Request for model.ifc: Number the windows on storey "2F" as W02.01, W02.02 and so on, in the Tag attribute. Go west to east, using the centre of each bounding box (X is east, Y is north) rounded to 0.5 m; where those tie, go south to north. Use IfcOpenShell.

First a look at what the model holds.

```python
import ifcopenshell
import ifcopenshell.util.element
import ifcopenshell.util.placement

model = ifcopenshell.open("model.ifc")
print(model.schema)
storey = next(s for s in model.by_type("IfcBuildingStorey") if s.Name == "2F")
windows = [e for e in ifcopenshell.util.element.get_decomposition(storey) if e.is_a("IfcWindow")]
for e in sorted(windows, key=lambda e: e.id()):
    origin = ifcopenshell.util.placement.get_local_placement(e.ObjectPlacement)[:3, 3]
    print(e.id(), e.Tag, e.Name, origin.round(2) + 0.0, sep=" | ")
```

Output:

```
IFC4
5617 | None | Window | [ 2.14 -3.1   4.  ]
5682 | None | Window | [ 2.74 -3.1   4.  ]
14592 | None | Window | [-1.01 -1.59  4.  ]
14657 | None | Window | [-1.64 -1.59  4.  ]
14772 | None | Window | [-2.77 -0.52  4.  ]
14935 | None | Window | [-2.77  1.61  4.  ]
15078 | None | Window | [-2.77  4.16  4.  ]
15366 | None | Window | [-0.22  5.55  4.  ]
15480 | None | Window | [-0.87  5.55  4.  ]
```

```python
import ifcopenshell
import ifcopenshell.geom
import ifcopenshell.util.element
import ifcopenshell.util.shape

model = ifcopenshell.open("model.ifc")
settings = ifcopenshell.geom.settings()
settings.set("use-world-coords", True)


def centre(element):
    shape = ifcopenshell.geom.create_shape(settings, element)
    return ifcopenshell.util.shape.get_bbox_centroid(shape.geometry)


storey = next(s for s in model.by_type("IfcBuildingStorey") if s.Name == "2F")
windows = [e for e in ifcopenshell.util.element.get_decomposition(storey) if e.is_a("IfcWindow")]

# Insertion points can sit at a corner or the storey origin, so sort by the geometry (in metres).
centres = {e: centre(e) for e in windows}
windows.sort(key=lambda e: (round(centres[e][0] / 0.5), centres[e][1]))

for i, e in enumerate(windows, start=1):
    number = f"W02.{i:02d}"
    e.Tag = number
    print(e.id(), number)

model.write("model_updated.ifc")
```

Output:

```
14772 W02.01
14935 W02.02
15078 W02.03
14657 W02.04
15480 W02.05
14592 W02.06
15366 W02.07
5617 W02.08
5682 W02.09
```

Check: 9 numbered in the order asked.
